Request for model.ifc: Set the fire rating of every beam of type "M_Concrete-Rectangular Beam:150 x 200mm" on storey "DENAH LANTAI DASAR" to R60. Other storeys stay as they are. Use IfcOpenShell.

First a look at what the model holds.

```python
import ifcopenshell
import ifcopenshell.util.element

model = ifcopenshell.open("model.ifc")
print(model.schema)
storey = next(s for s in model.by_type("IfcBuildingStorey") if s.Name == "DENAH LANTAI DASAR")
beams = [e for e in ifcopenshell.util.element.get_decomposition(storey) if e.is_a("IfcBeam")]
seen = {}
for e in beams:
    element_type = ifcopenshell.util.element.get_type(e)
    key = (element_type.Name if element_type != e and element_type else None, ifcopenshell.util.element.get_pset(e, "Pset_BeamCommon", "FireRating"))
    seen[key] = seen.get(key, 0) + 1
for (name, value), count in sorted(seen.items(), key=str):
    print(count, "x", name, "|", value)
```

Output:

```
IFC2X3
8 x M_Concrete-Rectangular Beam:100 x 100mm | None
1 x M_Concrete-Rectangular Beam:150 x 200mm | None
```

```python
import ifcopenshell
import ifcopenshell.api.pset
import ifcopenshell.util.element

model = ifcopenshell.open("model.ifc")

storey = next(s for s in model.by_type("IfcBuildingStorey") if s.Name == "DENAH LANTAI DASAR")
beams = [e for e in ifcopenshell.util.element.get_decomposition(storey) if e.is_a("IfcBeam")]

count = 0
for e in beams:
    element_type = ifcopenshell.util.element.get_type(e)
    if element_type in (None, e) or element_type.Name != "M_Concrete-Rectangular Beam:150 x 200mm":
        continue
    # add_pset returns the element's existing set when there is one.
    pset = ifcopenshell.api.pset.add_pset(model, product=e, name="Pset_BeamCommon")
    ifcopenshell.api.pset.edit_pset(model, pset=pset, properties={"FireRating": "R60"})
    count += 1

print(count, "beams updated")

model.write("model_updated.ifc")
```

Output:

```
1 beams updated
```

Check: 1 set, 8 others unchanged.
